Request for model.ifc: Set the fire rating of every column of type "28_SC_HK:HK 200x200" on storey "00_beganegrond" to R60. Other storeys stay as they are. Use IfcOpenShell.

First a look at what the model holds.

```python
import ifcopenshell
import ifcopenshell.util.element

model = ifcopenshell.open("model.ifc")
print(model.schema)
storey = next(s for s in model.by_type("IfcBuildingStorey") if s.Name == "00_beganegrond")
columns = [e for e in ifcopenshell.util.element.get_decomposition(storey) if e.is_a("IfcColumn")]
seen = {}
for e in columns:
    element_type = ifcopenshell.util.element.get_type(e)
    key = (element_type.Name if element_type != e and element_type else None, ifcopenshell.util.element.get_pset(e, "Pset_ColumnCommon", "FireRating"))
    seen[key] = seen.get(key, 0) + 1
for (name, value), count in sorted(seen.items(), key=str):
    print(count, "x", name, "|", value)
```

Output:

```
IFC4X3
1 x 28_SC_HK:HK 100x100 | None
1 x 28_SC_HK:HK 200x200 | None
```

```python
import ifcopenshell
import ifcopenshell.api.pset
import ifcopenshell.util.element

model = ifcopenshell.open("model.ifc")

storey = next(s for s in model.by_type("IfcBuildingStorey") if s.Name == "00_beganegrond")
columns = [e for e in ifcopenshell.util.element.get_decomposition(storey) if e.is_a("IfcColumn")]

count = 0
for e in columns:
    element_type = ifcopenshell.util.element.get_type(e)
    if element_type in (None, e) or element_type.Name != "28_SC_HK:HK 200x200":
        continue
    # add_pset returns the element's existing set when there is one.
    pset = ifcopenshell.api.pset.add_pset(model, product=e, name="Pset_ColumnCommon")
    ifcopenshell.api.pset.edit_pset(model, pset=pset, properties={"FireRating": "R60"})
    count += 1

print(count, "columns updated")

model.write("model-out.ifc")
```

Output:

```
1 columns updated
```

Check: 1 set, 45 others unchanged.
